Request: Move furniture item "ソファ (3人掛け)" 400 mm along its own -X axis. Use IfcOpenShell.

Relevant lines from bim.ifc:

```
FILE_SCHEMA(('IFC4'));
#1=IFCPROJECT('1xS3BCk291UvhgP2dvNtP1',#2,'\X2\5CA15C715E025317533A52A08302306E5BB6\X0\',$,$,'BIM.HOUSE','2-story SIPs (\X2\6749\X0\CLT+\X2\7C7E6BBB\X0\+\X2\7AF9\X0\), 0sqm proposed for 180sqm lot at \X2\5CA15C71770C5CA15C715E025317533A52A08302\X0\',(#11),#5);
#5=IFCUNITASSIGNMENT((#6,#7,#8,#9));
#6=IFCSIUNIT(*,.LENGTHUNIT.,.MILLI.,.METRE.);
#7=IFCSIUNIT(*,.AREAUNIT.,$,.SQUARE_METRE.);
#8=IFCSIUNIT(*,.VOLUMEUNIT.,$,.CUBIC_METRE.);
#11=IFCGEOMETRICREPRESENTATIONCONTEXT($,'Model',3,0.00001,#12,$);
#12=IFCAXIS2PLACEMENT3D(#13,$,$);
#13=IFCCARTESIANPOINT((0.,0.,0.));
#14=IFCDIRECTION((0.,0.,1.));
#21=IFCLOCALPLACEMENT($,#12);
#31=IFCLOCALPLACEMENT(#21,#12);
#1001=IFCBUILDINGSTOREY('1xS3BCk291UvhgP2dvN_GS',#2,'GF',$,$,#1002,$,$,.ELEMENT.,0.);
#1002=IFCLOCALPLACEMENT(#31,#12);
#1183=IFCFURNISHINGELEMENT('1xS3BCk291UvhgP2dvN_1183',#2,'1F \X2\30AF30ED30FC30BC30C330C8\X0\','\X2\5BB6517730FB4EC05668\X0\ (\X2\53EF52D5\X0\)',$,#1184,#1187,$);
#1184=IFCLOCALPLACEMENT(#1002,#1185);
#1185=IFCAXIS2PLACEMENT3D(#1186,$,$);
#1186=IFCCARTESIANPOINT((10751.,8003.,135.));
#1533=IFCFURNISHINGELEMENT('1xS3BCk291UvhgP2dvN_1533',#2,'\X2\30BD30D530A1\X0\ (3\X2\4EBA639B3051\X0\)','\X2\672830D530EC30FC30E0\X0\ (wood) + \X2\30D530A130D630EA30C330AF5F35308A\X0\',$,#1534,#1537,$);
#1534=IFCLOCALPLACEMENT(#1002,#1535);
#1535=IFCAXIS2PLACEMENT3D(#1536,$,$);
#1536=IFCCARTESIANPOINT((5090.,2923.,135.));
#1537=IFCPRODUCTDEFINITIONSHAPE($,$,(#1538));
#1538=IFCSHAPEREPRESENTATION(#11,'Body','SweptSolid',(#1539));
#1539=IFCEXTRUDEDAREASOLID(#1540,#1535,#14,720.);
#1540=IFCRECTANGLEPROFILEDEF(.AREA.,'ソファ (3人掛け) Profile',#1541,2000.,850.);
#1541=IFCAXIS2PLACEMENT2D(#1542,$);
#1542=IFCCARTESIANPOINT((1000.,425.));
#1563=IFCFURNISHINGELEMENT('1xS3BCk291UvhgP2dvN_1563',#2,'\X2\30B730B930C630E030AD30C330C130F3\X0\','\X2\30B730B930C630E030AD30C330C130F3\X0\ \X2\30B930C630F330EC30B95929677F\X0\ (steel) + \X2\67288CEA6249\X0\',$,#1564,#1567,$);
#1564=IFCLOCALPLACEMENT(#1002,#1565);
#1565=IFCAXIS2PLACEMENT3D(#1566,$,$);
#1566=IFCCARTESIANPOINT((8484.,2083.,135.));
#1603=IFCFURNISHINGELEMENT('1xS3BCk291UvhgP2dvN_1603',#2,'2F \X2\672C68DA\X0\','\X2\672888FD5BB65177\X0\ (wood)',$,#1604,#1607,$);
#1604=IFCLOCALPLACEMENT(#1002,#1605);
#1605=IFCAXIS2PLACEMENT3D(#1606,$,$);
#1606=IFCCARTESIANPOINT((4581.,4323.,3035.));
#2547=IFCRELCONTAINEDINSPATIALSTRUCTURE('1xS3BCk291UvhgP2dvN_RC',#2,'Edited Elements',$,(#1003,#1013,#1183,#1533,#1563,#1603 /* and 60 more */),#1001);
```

```python
import ifcopenshell
import ifcopenshell.api.geometry
import ifcopenshell.util.placement
import ifcopenshell.util.unit

model = ifcopenshell.open("bim.ifc")
unit_scale = ifcopenshell.util.unit.calculate_unit_scale(model)

item = model.by_id(1533)
matrix = ifcopenshell.util.placement.get_local_placement(item.ObjectPlacement)
matrix[:3, 3] -= matrix[:3, 0] * 0.4 / unit_scale
ifcopenshell.api.geometry.edit_object_placement(model, product=item, matrix=matrix, is_si=False)

print(ifcopenshell.util.placement.get_local_placement(item.ObjectPlacement).round(3) + 0.0)

model.write("bim-out.ifc")
```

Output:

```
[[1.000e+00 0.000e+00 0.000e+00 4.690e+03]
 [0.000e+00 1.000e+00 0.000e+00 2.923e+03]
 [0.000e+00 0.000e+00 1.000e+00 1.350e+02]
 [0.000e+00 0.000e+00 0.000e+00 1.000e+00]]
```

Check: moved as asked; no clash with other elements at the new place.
